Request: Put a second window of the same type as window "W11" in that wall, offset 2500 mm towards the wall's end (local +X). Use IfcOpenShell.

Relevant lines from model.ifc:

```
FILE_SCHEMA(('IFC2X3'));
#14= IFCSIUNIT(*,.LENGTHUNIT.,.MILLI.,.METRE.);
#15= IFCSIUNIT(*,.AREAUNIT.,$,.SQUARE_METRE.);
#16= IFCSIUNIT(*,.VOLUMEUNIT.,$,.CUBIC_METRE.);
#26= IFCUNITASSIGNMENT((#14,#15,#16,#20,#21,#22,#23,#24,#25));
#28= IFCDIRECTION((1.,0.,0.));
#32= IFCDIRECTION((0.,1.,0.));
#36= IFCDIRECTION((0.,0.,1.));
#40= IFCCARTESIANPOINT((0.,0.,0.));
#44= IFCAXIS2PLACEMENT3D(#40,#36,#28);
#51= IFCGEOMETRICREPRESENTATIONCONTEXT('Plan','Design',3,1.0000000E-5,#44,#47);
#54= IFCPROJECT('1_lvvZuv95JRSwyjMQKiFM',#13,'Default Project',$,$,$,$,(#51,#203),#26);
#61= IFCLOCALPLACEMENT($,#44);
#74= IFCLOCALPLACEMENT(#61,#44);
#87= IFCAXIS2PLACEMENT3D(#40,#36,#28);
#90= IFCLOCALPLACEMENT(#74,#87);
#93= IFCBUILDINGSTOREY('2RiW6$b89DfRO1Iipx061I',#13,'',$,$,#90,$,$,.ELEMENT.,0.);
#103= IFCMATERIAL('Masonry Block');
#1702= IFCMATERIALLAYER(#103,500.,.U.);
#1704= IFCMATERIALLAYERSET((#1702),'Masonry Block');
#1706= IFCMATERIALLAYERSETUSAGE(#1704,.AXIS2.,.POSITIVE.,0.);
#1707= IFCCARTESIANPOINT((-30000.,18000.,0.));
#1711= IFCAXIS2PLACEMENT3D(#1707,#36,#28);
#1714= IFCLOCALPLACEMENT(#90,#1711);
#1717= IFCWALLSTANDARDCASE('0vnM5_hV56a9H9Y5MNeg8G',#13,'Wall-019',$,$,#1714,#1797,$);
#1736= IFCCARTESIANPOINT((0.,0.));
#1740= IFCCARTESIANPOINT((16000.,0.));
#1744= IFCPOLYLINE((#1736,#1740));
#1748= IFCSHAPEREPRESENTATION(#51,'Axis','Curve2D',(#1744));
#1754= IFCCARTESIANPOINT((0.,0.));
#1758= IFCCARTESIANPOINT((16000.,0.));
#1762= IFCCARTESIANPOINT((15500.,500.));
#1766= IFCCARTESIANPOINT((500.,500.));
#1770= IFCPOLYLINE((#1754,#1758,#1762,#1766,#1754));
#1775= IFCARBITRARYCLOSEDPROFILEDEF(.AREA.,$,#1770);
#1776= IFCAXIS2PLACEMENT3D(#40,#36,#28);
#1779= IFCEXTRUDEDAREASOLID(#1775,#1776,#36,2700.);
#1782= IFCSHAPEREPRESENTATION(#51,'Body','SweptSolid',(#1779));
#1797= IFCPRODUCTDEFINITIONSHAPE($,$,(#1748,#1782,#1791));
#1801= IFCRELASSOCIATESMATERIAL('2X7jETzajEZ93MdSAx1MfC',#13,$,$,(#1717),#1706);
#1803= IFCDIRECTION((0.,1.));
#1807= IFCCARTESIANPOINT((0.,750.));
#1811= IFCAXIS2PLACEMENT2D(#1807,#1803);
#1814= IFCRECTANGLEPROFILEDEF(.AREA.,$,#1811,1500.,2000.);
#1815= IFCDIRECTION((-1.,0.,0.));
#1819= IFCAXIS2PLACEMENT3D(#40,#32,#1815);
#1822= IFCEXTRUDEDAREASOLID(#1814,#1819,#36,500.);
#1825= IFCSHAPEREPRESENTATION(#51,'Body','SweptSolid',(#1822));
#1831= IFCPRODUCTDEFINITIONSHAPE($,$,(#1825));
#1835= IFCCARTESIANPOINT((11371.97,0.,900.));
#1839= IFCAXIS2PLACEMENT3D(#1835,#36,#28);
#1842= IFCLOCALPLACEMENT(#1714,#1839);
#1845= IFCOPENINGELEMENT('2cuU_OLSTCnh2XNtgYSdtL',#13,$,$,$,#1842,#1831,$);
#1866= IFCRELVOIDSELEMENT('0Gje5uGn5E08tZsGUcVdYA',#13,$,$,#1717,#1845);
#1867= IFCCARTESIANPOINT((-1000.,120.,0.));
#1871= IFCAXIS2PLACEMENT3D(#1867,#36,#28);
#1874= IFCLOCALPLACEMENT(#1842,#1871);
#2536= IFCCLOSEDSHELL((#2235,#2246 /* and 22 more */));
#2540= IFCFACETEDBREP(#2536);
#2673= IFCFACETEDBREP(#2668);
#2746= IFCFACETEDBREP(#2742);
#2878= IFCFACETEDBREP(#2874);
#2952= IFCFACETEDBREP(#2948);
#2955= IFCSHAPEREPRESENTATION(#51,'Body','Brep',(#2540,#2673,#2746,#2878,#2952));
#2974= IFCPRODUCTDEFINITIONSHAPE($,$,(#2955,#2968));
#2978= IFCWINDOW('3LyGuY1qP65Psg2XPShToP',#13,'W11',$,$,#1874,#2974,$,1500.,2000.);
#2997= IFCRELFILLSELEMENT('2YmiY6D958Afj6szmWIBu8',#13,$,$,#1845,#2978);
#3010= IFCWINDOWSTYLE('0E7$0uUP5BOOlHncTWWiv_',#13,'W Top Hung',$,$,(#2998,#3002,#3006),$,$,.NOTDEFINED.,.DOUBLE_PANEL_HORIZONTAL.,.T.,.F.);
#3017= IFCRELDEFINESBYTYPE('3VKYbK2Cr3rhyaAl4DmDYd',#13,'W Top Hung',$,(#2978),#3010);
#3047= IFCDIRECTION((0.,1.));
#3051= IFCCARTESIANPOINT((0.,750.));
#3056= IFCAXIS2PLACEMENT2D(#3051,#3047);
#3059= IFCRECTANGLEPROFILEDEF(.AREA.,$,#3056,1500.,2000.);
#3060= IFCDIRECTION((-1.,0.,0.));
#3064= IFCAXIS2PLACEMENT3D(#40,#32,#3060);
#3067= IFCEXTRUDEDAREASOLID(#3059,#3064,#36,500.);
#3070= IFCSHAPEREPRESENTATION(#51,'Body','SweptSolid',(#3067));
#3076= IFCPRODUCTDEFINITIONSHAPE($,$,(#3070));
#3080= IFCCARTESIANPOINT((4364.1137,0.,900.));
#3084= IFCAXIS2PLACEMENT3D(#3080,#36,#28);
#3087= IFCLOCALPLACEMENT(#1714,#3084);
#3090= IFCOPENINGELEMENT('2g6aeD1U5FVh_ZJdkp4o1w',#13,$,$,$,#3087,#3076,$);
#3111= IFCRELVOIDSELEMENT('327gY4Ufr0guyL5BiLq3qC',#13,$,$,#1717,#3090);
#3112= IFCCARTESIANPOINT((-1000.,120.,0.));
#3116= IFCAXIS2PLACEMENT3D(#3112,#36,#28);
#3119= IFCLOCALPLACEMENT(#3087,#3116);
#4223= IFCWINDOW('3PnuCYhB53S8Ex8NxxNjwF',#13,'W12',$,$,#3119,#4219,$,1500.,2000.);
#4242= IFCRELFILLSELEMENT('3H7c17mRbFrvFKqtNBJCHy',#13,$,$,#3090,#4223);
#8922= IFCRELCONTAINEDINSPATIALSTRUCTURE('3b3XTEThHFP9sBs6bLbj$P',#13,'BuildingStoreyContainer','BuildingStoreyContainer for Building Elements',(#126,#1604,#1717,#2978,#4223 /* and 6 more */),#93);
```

```python
import ifcopenshell
import ifcopenshell.api.feature
import ifcopenshell.api.geometry
import ifcopenshell.api.root
import ifcopenshell.geom
import ifcopenshell.util.element
import ifcopenshell.util.placement
import ifcopenshell.util.shape

model = ifcopenshell.open("model.ifc")
settings = ifcopenshell.geom.settings()


def volume(element):
    """Net volume in cubic metres, openings subtracted."""
    shape = ifcopenshell.geom.create_shape(settings, element)
    return ifcopenshell.util.shape.get_volume(shape.geometry)


def reuse_history(source, copy):
    """copy_class also copies each property set's owner history, people and application; keep the originals."""
    for rel in copy.IsDefinedBy:
        if rel.is_a("IfcRelDefinesByProperties") and (history := rel.RelatingPropertyDefinition.OwnerHistory):
            rel.RelatingPropertyDefinition.OwnerHistory = source.OwnerHistory
            ifcopenshell.util.element.remove_deep2(model, history)


window = model.by_id(2978)
opening = window.FillsVoids[0].RelatingOpeningElement
wall = opening.VoidsElements[0].RelatingBuildingElement
before = volume(wall)
shift = ifcopenshell.util.placement.get_local_placement(wall.ObjectPlacement)[:3, 0] * 2500.0

# copy_class copies the void relationship, type, container and properties, but no geometry.
new_opening = ifcopenshell.api.root.copy_class(model, product=opening)
new_opening.Representation = ifcopenshell.util.element.copy_deep(
    model, opening.Representation, exclude=["IfcGeometricRepresentationContext", "IfcRepresentationMap"]
)
new_window = ifcopenshell.api.root.copy_class(model, product=window)
new_window.Representation = ifcopenshell.util.element.copy_deep(
    model, window.Representation, exclude=["IfcGeometricRepresentationContext", "IfcRepresentationMap"]
)
reuse_history(window, new_window)
fills = ifcopenshell.api.feature.add_filling(model, opening=new_opening, element=new_window)
fills.OwnerHistory = new_window.OwnerHistory  # required in IFC2X3

for old, new in ((opening, new_opening), (window, new_window)):
    matrix = ifcopenshell.util.placement.get_local_placement(old.ObjectPlacement)
    matrix[:3, 3] += shift
    ifcopenshell.api.geometry.edit_object_placement(model, product=new, matrix=matrix, is_si=False)

after = volume(wall)

print(f"wall volume {before:.3f} -> {after:.3f} m3")

model.write("model-out.ifc")
```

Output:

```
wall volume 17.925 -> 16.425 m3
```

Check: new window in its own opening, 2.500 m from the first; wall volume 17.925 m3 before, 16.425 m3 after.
